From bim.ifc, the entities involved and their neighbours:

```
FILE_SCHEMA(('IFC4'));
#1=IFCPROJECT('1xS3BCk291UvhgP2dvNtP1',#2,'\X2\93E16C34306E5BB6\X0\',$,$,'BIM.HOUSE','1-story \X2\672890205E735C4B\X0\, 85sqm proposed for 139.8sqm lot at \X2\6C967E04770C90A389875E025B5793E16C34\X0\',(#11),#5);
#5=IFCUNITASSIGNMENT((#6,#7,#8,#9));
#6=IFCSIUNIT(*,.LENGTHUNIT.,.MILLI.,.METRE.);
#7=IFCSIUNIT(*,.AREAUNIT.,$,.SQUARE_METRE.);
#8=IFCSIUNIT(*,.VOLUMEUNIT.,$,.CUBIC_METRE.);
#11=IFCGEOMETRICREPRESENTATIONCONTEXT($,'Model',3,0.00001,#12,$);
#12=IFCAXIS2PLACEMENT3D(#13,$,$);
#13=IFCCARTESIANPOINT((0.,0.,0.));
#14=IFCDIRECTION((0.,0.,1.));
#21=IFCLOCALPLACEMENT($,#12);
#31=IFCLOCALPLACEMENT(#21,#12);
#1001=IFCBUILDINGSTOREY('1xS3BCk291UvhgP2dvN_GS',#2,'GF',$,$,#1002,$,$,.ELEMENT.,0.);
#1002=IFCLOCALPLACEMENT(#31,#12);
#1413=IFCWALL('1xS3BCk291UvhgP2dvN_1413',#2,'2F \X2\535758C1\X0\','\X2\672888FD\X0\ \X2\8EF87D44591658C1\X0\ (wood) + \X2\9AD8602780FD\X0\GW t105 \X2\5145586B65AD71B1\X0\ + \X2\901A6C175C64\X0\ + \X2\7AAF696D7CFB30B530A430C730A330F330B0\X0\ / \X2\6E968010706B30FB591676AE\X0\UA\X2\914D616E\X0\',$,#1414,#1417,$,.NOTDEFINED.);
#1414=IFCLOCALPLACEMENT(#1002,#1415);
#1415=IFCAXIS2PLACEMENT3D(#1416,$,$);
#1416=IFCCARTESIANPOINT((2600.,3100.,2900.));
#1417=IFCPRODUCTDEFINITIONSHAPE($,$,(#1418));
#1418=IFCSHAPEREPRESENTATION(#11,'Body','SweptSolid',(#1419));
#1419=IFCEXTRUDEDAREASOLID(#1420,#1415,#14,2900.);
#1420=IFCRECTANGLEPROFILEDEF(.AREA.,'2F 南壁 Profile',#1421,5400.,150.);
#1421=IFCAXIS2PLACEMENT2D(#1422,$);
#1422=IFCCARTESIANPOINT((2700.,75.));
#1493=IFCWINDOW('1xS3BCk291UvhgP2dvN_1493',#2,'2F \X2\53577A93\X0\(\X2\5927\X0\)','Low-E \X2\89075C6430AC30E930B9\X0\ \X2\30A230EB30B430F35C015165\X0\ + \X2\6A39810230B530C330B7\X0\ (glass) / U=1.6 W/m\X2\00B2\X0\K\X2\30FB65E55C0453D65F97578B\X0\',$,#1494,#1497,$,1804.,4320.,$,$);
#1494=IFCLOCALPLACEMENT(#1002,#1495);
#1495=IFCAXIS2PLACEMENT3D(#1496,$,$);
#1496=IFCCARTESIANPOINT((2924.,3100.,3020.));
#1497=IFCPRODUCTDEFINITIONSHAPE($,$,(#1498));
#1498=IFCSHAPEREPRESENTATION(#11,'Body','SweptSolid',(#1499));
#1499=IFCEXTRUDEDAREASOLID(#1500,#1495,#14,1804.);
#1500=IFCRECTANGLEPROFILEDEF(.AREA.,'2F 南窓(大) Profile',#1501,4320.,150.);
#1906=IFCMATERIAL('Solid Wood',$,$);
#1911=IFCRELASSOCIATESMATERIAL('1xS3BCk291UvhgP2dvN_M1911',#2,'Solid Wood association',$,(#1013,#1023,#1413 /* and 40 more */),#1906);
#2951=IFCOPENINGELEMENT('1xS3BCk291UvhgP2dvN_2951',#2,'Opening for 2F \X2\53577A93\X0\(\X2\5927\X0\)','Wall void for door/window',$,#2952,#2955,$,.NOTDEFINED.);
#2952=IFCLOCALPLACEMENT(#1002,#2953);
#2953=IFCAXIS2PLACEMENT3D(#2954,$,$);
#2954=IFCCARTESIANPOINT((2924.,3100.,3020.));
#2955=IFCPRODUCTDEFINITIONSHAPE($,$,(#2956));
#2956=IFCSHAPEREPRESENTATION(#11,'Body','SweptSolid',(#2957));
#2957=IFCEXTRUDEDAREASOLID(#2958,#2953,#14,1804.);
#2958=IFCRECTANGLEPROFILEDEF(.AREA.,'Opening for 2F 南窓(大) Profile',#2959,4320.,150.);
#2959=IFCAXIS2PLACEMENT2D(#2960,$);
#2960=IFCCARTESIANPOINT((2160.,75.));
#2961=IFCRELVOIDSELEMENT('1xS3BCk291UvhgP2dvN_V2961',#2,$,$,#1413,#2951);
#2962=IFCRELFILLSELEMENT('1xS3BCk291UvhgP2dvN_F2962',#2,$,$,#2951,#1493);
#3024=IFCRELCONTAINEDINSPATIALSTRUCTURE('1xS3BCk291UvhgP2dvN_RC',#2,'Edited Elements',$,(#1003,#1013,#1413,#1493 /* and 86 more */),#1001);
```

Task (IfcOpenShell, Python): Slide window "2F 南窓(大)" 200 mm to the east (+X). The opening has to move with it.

```python
import ifcopenshell
import ifcopenshell.api.geometry
import ifcopenshell.util.placement

model = ifcopenshell.open("bim.ifc")

window = model.by_guid("1xS3BCk291UvhgP2dvN_1493")
opening = window.FillsVoids[0].RelatingOpeningElement
wall = opening.VoidsElements[0].RelatingBuildingElement

wall_matrix = ifcopenshell.util.placement.get_local_placement(wall.ObjectPlacement)
shift = wall_matrix[:3, 0] * 200.0
before = ifcopenshell.util.placement.get_local_placement(window.ObjectPlacement)[:3, 3].copy()

# The window is not placed relative to its opening, so move both.
for product in (opening, window):
    matrix = ifcopenshell.util.placement.get_local_placement(product.ObjectPlacement)
    matrix[:3, 3] += shift
    ifcopenshell.api.geometry.edit_object_placement(model, product=product, matrix=matrix, is_si=False)

after = ifcopenshell.util.placement.get_local_placement(window.ObjectPlacement)[:3, 3]
print("window moved by", (after - before).round(3) + 0.0)

model.write("bim-out.ifc")
```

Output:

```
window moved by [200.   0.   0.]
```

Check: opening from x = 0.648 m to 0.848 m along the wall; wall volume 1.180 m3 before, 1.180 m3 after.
